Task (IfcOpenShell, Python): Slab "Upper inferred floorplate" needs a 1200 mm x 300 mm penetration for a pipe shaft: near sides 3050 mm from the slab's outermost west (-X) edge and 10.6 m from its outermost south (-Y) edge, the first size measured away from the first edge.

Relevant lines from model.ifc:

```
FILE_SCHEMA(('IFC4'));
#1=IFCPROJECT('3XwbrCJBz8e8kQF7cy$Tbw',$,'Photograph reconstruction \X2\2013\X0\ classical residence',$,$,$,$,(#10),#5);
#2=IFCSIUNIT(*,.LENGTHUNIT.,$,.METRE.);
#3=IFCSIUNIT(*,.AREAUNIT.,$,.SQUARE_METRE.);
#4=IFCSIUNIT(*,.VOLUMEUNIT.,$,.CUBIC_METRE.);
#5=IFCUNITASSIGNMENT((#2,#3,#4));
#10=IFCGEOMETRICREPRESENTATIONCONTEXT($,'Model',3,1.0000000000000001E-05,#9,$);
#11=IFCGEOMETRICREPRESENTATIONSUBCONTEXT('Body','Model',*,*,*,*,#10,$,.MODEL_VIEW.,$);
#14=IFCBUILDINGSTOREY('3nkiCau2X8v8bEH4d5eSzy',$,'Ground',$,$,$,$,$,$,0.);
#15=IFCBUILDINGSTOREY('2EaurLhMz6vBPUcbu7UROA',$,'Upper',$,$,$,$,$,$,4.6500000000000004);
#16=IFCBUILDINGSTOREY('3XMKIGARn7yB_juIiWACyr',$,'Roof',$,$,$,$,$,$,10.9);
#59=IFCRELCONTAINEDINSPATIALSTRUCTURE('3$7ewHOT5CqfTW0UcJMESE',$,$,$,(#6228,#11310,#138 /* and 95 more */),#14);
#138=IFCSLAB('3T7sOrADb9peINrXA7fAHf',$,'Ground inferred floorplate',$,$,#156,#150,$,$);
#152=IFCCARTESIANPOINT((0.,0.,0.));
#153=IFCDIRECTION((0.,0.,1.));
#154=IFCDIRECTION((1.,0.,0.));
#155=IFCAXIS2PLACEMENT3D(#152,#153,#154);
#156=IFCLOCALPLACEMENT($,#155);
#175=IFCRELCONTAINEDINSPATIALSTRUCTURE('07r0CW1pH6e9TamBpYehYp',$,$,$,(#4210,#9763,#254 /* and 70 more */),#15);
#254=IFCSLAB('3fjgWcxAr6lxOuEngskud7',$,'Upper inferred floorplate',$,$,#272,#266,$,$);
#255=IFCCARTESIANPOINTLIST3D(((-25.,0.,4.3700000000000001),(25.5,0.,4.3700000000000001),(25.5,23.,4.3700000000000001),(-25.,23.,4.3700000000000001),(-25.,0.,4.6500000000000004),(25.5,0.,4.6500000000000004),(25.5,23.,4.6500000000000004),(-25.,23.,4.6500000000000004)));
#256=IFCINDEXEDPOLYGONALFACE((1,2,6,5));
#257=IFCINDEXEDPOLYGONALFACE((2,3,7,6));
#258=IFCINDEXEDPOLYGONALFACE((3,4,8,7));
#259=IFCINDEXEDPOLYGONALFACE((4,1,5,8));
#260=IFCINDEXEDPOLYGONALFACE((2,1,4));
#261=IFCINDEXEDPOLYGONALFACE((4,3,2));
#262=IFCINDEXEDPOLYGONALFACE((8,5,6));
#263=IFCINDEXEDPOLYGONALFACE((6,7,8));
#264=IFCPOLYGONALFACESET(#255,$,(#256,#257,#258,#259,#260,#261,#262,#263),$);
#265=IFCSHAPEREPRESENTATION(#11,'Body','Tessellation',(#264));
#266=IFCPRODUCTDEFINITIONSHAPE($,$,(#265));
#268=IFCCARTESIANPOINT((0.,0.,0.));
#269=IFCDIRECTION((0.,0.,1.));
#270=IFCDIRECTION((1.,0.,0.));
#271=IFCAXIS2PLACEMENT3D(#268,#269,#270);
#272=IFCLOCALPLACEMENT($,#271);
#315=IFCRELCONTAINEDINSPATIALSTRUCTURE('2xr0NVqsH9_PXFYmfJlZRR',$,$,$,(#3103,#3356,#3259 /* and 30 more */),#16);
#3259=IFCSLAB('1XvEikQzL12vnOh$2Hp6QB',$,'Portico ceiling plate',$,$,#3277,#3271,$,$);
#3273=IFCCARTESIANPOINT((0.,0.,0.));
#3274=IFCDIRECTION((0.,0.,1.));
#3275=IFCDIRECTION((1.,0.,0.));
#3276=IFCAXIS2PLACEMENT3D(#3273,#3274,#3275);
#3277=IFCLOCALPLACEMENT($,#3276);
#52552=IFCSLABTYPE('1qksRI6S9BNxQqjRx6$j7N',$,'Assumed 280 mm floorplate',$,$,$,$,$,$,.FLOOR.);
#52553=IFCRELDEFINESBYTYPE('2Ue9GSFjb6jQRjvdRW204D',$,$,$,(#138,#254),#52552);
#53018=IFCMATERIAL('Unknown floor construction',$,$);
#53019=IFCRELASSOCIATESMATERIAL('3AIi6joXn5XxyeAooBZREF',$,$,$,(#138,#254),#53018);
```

```python
import numpy as np
import ifcopenshell
import ifcopenshell.api.feature
import ifcopenshell.api.geometry
import ifcopenshell.api.root
import ifcopenshell.geom
import ifcopenshell.util.placement
import ifcopenshell.util.representation
import ifcopenshell.util.shape
import ifcopenshell.util.unit

model = ifcopenshell.open("model.ifc")
unit_scale = ifcopenshell.util.unit.calculate_unit_scale(model)
settings = ifcopenshell.geom.settings()


def volume(element):
    """Net volume in cubic metres, openings subtracted."""
    shape = ifcopenshell.geom.create_shape(settings, element)
    return ifcopenshell.util.shape.get_volume(shape.geometry)


slab = model.by_id(254)
before = volume(slab)

# Extent in the slab's own axes, in metres. The edges named are its -X and -Y sides.
slab_shape = ifcopenshell.geom.create_shape(settings, slab)
vertices = ifcopenshell.util.shape.get_vertices(slab_shape.geometry)
x_min, y_min, bottom = vertices.min(axis=0)
top = vertices[:, 2].max()

opening = ifcopenshell.api.root.create_entity(model, ifc_class="IfcOpeningElement", name="Pipe shaft opening", predefined_type="OPENING")
context = ifcopenshell.util.representation.get_context(model, "Model", "Body", "MODEL_VIEW")
width, depth = 1.2, 0.3
outline = [(0.0, 0.0), (width, 0.0), (width, depth), (0.0, depth), (0.0, 0.0)]
# Overshoot both faces by 50 mm so the cut is clean.
shape = ifcopenshell.api.geometry.add_slab_representation(
    model, context=context, depth=top - bottom + 0.1, polyline=outline
)
ifcopenshell.api.geometry.assign_representation(model, product=opening, representation=shape)

matrix = ifcopenshell.util.placement.get_local_placement(slab.ObjectPlacement)
matrix[:, 3] = matrix @ np.append(np.array([x_min + 3.05, y_min + 10.6, bottom - 0.05]) / unit_scale, 1.0)
ifcopenshell.api.geometry.edit_object_placement(model, product=opening, matrix=matrix, is_si=False)
ifcopenshell.api.feature.add_feature(model, feature=opening, element=slab)

after = volume(slab)

print(f"slab volume {before:.3f} -> {after:.3f} m3")

model.write("model_edited.ifc")
```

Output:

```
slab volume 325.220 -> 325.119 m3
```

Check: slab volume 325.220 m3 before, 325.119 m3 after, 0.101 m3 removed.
